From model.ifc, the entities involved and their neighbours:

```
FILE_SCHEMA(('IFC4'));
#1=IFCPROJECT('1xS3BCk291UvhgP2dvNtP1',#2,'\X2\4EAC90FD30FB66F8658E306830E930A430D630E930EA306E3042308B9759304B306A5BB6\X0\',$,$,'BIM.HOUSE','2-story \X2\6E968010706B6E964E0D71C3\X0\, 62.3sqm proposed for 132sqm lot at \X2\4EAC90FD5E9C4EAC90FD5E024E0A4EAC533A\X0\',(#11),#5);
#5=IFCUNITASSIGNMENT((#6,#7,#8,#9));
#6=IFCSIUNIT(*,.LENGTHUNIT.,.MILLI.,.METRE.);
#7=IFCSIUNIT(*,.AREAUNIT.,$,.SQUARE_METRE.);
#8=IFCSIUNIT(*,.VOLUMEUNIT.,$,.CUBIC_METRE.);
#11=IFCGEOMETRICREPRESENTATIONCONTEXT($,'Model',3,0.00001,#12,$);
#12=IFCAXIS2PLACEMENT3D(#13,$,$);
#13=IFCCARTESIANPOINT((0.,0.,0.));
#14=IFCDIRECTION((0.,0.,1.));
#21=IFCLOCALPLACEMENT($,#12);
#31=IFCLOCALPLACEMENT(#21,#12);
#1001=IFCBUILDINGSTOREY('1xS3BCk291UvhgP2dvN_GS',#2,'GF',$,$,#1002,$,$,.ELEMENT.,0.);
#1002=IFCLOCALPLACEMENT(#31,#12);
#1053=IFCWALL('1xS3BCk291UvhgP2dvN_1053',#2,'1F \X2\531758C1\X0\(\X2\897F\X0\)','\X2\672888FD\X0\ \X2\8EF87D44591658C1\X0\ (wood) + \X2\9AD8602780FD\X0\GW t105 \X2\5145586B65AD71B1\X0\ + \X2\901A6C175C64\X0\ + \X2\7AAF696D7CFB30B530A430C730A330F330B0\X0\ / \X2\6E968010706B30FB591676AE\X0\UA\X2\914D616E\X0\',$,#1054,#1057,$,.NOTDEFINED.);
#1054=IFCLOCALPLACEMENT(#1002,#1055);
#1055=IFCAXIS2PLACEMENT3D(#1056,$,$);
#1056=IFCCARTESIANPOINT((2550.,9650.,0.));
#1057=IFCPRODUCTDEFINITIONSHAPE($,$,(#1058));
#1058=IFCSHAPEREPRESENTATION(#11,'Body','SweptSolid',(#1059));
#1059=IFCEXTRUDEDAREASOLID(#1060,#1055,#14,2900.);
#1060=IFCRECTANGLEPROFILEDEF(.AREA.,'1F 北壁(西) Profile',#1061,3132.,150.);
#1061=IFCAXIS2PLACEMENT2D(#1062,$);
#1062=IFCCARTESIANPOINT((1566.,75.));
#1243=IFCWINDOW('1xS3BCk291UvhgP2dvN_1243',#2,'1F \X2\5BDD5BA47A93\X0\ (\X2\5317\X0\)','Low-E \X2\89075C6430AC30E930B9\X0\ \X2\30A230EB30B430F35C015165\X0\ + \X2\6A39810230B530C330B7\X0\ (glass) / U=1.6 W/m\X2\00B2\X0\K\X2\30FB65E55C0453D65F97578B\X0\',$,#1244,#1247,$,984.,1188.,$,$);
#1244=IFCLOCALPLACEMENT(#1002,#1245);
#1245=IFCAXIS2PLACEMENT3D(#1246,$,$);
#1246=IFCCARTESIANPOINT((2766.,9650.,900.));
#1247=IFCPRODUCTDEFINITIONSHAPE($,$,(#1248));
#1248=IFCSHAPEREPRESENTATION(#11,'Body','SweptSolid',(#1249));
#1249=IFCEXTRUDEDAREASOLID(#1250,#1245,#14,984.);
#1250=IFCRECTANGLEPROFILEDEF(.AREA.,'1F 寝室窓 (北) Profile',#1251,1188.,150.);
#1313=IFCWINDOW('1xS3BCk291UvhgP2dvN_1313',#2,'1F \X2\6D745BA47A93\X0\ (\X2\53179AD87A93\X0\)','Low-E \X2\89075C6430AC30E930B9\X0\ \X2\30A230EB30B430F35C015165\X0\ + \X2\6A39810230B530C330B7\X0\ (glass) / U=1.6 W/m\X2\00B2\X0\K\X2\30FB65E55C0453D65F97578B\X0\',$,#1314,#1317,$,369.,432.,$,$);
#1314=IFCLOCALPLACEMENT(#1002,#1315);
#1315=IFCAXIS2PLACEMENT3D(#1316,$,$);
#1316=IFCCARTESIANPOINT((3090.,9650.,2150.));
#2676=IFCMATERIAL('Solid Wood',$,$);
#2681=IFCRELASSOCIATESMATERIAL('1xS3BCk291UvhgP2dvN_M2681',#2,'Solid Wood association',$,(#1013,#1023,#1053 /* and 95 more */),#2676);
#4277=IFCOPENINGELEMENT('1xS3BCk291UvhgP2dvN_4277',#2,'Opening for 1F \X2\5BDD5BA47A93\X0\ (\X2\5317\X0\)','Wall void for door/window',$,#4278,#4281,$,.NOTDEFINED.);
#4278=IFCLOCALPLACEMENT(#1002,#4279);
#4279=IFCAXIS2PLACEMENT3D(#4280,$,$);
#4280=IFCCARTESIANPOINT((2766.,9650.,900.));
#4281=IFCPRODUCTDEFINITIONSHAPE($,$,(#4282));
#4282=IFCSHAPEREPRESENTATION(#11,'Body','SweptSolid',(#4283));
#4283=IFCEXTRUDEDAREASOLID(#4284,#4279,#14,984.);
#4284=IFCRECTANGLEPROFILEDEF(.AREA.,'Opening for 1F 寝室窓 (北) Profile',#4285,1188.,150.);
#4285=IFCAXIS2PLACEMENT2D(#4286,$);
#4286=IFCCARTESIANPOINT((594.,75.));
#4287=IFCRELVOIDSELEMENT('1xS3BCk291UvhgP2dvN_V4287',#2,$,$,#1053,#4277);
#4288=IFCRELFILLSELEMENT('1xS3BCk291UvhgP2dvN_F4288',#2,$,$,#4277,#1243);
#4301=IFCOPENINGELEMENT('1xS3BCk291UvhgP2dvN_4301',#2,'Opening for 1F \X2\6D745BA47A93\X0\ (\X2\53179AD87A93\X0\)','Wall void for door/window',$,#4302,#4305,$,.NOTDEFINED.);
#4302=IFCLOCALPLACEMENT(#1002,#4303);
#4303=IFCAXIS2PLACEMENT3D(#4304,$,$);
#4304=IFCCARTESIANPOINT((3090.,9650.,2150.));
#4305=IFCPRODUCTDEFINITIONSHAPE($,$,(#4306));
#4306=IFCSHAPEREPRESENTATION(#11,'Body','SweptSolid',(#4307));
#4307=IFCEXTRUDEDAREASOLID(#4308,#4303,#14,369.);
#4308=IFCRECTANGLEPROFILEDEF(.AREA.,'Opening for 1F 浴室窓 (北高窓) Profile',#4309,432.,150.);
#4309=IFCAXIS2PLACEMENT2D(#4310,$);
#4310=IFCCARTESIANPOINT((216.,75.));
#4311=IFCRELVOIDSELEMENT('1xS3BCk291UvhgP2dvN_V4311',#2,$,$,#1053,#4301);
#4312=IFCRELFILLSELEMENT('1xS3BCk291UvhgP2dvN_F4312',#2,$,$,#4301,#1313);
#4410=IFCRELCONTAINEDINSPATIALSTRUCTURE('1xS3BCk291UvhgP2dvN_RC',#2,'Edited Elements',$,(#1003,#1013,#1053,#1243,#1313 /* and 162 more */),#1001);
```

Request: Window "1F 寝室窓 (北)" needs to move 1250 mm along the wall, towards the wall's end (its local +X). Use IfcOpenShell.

```python
import ifcopenshell
import ifcopenshell.api.geometry
import ifcopenshell.util.placement
import ifcopenshell.util.unit

model = ifcopenshell.open("model.ifc")
unit_scale = ifcopenshell.util.unit.calculate_unit_scale(model)

window = model.by_guid("1xS3BCk291UvhgP2dvN_1243")
opening = window.FillsVoids[0].RelatingOpeningElement
wall = opening.VoidsElements[0].RelatingBuildingElement

wall_matrix = ifcopenshell.util.placement.get_local_placement(wall.ObjectPlacement)
shift = wall_matrix[:3, 0] * 1.25 / unit_scale
before = ifcopenshell.util.placement.get_local_placement(window.ObjectPlacement)[:3, 3].copy()

# The window is not placed relative to its opening, so move both.
for product in (opening, window):
    matrix = ifcopenshell.util.placement.get_local_placement(product.ObjectPlacement)
    matrix[:3, 3] += shift
    ifcopenshell.api.geometry.edit_object_placement(model, product=product, matrix=matrix, is_si=False)

after = ifcopenshell.util.placement.get_local_placement(window.ObjectPlacement)[:3, 3]
print("window moved by", (after - before).round(3) + 0.0)

model.write("model-out.ifc")
```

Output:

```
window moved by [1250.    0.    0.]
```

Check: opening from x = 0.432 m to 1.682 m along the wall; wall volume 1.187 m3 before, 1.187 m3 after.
